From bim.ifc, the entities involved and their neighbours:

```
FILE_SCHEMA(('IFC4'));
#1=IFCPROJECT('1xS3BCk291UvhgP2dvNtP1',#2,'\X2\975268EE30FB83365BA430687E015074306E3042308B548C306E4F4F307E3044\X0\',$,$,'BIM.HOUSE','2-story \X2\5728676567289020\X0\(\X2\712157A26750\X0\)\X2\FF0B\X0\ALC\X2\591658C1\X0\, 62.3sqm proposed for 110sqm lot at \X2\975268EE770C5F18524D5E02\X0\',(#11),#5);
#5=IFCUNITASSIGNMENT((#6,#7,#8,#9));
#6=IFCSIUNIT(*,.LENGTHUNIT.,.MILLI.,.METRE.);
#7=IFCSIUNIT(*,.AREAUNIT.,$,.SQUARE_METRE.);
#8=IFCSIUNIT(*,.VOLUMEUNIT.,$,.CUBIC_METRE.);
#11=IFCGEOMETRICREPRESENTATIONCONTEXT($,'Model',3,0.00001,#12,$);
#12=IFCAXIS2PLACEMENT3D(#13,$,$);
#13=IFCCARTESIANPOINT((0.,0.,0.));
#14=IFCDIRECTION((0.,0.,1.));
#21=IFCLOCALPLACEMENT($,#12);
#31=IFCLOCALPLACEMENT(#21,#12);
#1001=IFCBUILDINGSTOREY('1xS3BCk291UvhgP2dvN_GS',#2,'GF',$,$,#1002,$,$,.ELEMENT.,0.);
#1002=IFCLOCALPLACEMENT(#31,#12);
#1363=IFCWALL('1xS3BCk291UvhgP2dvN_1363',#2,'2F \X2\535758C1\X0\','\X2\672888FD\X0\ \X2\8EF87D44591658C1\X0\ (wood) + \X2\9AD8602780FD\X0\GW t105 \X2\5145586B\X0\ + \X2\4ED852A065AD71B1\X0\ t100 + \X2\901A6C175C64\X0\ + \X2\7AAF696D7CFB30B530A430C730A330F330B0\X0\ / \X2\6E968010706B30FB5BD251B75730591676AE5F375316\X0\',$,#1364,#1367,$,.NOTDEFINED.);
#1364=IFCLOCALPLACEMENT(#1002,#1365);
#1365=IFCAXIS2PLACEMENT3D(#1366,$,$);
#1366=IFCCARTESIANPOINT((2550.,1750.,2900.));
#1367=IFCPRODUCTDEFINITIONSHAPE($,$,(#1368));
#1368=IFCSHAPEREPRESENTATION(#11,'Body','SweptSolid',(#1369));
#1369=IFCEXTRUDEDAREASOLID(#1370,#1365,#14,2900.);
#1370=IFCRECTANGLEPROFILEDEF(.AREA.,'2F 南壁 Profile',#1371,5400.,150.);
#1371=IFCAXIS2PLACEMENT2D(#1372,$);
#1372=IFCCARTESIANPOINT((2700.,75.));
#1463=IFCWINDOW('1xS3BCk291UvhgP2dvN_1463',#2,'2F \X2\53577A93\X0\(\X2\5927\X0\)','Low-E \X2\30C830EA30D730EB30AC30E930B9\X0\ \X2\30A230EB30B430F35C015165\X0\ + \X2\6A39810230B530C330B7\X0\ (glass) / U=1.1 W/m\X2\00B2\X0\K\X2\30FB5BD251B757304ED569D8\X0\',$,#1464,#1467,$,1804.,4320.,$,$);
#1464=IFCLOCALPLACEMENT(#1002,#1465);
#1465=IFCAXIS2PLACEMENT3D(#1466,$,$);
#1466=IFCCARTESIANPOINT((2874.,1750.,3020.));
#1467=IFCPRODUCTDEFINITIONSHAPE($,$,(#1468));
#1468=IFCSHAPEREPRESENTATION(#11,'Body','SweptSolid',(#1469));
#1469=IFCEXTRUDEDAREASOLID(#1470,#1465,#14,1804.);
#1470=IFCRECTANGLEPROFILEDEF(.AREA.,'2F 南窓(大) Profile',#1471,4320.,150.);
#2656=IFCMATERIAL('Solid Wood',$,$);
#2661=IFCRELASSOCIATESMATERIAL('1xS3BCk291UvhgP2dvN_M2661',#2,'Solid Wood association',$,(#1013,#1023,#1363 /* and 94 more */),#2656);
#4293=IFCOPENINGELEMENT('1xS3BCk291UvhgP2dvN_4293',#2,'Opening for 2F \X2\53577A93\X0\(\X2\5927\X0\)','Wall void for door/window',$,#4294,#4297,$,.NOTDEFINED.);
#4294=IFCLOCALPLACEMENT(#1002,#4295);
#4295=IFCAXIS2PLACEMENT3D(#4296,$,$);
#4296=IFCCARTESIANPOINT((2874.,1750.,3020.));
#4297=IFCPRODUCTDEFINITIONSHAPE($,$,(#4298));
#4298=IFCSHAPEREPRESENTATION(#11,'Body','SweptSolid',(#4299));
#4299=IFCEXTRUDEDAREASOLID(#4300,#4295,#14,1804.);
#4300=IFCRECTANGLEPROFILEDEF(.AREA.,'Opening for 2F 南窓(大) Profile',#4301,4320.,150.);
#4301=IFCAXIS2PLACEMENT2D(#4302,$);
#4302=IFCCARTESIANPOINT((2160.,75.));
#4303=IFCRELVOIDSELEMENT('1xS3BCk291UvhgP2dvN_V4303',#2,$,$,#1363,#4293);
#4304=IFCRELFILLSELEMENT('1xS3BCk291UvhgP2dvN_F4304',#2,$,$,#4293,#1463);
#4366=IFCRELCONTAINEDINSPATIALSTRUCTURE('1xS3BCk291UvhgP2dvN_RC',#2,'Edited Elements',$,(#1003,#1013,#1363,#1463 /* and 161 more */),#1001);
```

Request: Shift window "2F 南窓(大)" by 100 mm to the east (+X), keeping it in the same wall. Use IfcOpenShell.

```python
import ifcopenshell
import ifcopenshell.api.geometry
import ifcopenshell.util.placement
import ifcopenshell.util.unit

model = ifcopenshell.open("bim.ifc")
unit_scale = ifcopenshell.util.unit.calculate_unit_scale(model)

window = model.by_guid("1xS3BCk291UvhgP2dvN_1463")
opening = window.FillsVoids[0].RelatingOpeningElement
wall = opening.VoidsElements[0].RelatingBuildingElement

wall_matrix = ifcopenshell.util.placement.get_local_placement(wall.ObjectPlacement)
shift = wall_matrix[:3, 0] * 0.1 / unit_scale
before = ifcopenshell.util.placement.get_local_placement(window.ObjectPlacement)[:3, 3].copy()

# The window is not placed relative to its opening, so move both.
for product in (opening, window):
    matrix = ifcopenshell.util.placement.get_local_placement(product.ObjectPlacement)
    matrix[:3, 3] += shift
    ifcopenshell.api.geometry.edit_object_placement(model, product=product, matrix=matrix, is_si=False)

after = ifcopenshell.util.placement.get_local_placement(window.ObjectPlacement)[:3, 3]
print("window moved by", (after - before).round(3) + 0.0)

model.write("bim_rev.ifc")
```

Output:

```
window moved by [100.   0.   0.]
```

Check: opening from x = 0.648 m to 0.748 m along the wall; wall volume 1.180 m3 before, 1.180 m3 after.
